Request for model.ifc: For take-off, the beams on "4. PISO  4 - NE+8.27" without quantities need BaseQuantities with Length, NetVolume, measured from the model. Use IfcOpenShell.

First a look at what the model holds.

```python
import ifcopenshell
import ifcopenshell.util.element
import ifcopenshell.util.unit

model = ifcopenshell.open("model.ifc")
print(model.schema)
for unit_type in ("LENGTHUNIT", "AREAUNIT", "VOLUMEUNIT"):
    print(unit_type, ifcopenshell.util.unit.calculate_unit_scale(model, unit_type))
storey = next(s for s in model.by_type("IfcBuildingStorey") if s.Name == "4. PISO  4 - NE+8.27")
beams = [e for e in ifcopenshell.util.element.get_decomposition(storey) if e.is_a("IfcBeam")]
for e in sorted(beams, key=lambda e: e.id()):
    print(e.id(), e.is_a(), e.Name, list(ifcopenshell.util.element.get_psets(e, qtos_only=True)), sep=" | ")
```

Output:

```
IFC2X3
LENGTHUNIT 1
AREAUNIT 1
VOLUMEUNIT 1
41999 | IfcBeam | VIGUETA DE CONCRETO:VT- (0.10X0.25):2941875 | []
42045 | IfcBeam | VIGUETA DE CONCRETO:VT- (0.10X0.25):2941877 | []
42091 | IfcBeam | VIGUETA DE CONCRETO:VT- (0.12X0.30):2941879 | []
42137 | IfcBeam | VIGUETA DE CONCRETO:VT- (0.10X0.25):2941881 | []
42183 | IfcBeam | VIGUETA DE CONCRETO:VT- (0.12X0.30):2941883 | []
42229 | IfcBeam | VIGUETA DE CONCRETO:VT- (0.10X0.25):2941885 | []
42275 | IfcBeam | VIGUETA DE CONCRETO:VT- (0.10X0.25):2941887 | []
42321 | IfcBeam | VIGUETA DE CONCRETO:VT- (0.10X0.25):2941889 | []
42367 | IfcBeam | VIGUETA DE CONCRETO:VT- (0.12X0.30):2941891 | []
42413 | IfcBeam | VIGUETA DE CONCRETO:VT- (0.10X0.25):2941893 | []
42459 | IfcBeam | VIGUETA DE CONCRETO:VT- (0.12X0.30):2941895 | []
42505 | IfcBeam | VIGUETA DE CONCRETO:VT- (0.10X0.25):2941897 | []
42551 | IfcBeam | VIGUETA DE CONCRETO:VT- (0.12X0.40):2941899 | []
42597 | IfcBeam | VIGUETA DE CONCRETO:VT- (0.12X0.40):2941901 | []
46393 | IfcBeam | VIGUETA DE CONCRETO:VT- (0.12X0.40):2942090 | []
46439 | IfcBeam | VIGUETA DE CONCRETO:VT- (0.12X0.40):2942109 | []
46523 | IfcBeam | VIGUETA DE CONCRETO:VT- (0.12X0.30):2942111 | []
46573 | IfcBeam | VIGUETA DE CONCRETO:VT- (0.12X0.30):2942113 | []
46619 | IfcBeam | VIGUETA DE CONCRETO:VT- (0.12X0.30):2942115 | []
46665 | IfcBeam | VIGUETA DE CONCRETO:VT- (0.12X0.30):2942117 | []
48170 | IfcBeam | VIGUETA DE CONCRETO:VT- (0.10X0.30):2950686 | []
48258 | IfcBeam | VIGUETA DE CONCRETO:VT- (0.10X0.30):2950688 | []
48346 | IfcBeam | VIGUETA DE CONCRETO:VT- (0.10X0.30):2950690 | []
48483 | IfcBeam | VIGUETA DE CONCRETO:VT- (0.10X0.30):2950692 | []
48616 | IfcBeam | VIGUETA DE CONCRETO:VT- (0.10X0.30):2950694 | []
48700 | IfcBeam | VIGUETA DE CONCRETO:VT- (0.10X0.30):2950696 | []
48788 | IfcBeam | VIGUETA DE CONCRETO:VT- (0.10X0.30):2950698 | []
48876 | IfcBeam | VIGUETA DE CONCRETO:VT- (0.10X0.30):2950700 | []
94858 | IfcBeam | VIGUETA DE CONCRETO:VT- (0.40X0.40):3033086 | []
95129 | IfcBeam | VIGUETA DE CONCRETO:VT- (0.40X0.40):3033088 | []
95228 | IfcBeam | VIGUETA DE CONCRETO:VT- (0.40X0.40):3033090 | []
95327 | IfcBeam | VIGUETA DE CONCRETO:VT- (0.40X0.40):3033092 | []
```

```python
import ifcopenshell
import ifcopenshell.api.pset
import ifcopenshell.geom
import ifcopenshell.util.element
import ifcopenshell.util.shape
import ifcopenshell.util.unit

model = ifcopenshell.open("model.ifc")
unit_scale = ifcopenshell.util.unit.calculate_unit_scale(model)
volume_scale = ifcopenshell.util.unit.calculate_unit_scale(model, "VOLUMEUNIT")
settings = ifcopenshell.geom.settings()

storey = next(s for s in model.by_type("IfcBuildingStorey") if s.Name == "4. PISO  4 - NE+8.27")
beams = [e for e in ifcopenshell.util.element.get_decomposition(storey) if e.is_a("IfcBeam")]

for e in sorted(beams, key=lambda e: e.id()):
    if ifcopenshell.util.element.get_psets(e, qtos_only=True, should_inherit=False):
        continue
    # Geometry comes back in metres, in the element's own axes.
    shape = ifcopenshell.geom.create_shape(settings, e)
    values = {
        "Length": ifcopenshell.util.shape.get_max_xyz(shape.geometry) / unit_scale,
        "NetVolume": ifcopenshell.util.shape.get_volume(shape.geometry) / volume_scale,
    }
    qto = ifcopenshell.api.pset.add_qto(model, product=e, name="BaseQuantities")
    ifcopenshell.api.pset.edit_qto(model, qto=qto, properties=values)
    print(e.id(), {k: round(v, 3) for k, v in values.items()})

model.write("model_v2.ifc")
```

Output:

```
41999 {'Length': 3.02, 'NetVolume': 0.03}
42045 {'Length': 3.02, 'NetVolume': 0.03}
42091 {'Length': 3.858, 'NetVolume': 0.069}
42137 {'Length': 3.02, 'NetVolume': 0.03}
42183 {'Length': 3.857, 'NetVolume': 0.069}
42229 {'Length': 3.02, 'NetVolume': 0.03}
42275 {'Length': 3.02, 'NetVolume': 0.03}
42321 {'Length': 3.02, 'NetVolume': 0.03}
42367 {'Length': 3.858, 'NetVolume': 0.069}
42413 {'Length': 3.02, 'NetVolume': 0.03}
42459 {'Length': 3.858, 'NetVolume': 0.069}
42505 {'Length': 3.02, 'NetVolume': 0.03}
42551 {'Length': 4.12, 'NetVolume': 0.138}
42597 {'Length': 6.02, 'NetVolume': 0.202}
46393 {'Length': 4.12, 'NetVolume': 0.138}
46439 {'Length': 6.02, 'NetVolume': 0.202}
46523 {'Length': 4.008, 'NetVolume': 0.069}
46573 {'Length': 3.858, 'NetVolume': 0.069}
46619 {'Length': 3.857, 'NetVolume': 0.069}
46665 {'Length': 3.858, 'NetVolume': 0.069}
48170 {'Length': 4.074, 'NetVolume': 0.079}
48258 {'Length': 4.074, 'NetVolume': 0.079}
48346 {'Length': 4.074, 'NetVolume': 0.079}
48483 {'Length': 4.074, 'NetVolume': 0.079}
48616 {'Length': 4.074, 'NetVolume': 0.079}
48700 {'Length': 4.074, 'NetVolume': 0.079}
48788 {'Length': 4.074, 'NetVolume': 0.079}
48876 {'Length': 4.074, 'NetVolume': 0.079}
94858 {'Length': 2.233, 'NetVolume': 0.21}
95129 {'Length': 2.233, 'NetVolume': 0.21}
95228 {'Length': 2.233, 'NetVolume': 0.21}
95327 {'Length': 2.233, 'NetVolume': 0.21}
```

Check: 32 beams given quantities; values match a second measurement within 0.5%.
